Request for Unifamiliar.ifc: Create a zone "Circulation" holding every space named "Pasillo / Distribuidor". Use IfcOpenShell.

First a look at what the model holds.

```python
import ifcopenshell

model = ifcopenshell.open("Unifamiliar.ifc")
print(model.schema)
seen = {}
for space in model.by_type("IfcSpace"):
    seen[space.LongName] = seen.get(space.LongName, 0) + 1
for name, count in sorted(seen.items(), key=str):
    print(count, "x", name)
print("zones:", [z.Name for z in model.by_type("IfcZone")][:20])
```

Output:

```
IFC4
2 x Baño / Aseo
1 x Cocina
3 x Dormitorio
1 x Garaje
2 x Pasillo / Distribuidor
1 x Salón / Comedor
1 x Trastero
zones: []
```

```python
import ifcopenshell
import ifcopenshell.api.group
import ifcopenshell.api.root

model = ifcopenshell.open("Unifamiliar.ifc")

names = {"Pasillo / Distribuidor"}
spaces = [s for s in model.by_type("IfcSpace") if s.LongName in names]

zone = ifcopenshell.api.root.create_entity(model, ifc_class="IfcZone", name="Circulation")
ifcopenshell.api.group.assign_group(model, products=spaces, group=zone)
print(len(spaces), "spaces in", zone.Name)

model.write("Unifamiliar_updated.ifc")
```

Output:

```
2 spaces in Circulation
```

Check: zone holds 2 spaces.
